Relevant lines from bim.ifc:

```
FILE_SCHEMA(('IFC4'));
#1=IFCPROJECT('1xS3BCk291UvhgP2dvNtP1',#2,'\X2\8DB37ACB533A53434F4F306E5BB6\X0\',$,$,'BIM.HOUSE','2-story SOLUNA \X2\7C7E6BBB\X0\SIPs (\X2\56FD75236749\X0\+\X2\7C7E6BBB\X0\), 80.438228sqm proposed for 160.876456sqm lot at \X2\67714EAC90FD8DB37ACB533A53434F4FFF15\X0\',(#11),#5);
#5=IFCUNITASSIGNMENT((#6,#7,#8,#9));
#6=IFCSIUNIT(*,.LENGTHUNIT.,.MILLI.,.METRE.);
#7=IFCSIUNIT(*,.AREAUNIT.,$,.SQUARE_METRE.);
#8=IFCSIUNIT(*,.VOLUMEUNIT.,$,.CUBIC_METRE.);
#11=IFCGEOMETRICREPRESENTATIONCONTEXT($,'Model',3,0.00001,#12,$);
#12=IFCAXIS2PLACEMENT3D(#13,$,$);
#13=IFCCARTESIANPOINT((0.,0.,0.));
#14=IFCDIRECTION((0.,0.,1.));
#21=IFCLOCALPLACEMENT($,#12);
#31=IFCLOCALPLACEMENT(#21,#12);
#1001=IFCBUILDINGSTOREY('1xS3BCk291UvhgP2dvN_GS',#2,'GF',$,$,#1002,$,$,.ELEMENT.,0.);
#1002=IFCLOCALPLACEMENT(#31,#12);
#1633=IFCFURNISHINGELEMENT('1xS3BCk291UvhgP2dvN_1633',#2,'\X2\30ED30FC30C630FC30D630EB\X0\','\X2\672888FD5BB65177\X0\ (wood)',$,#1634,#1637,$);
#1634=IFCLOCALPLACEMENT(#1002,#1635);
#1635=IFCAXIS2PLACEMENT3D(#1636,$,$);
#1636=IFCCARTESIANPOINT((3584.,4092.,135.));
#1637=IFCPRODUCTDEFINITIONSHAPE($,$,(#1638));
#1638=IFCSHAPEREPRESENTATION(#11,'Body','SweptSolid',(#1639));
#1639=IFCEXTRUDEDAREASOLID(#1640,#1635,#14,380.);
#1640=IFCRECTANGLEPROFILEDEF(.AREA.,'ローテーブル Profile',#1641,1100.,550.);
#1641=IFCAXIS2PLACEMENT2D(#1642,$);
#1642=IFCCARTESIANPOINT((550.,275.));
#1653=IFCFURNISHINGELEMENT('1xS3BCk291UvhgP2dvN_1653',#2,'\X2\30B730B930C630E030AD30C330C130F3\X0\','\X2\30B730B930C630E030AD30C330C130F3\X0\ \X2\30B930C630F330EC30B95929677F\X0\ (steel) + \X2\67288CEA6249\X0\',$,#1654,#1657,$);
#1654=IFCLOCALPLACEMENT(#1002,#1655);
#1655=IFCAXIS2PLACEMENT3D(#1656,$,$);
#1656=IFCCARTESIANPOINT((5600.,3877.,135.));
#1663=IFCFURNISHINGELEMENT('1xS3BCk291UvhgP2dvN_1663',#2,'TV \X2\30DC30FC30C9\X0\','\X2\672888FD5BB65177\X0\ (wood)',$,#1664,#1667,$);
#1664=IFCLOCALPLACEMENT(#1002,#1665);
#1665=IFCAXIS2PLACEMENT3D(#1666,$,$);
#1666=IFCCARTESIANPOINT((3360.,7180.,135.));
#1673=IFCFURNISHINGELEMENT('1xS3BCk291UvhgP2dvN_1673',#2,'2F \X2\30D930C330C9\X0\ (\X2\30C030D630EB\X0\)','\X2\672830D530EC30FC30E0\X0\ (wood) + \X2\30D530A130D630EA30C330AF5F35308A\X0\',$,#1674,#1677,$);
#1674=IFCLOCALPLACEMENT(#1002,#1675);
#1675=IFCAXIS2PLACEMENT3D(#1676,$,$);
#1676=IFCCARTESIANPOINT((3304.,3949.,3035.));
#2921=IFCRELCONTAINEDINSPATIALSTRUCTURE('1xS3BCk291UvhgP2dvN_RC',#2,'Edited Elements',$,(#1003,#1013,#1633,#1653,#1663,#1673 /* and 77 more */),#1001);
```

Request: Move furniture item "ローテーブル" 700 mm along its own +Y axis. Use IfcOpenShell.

```python
import ifcopenshell
import ifcopenshell.api.geometry
import ifcopenshell.util.placement
import ifcopenshell.util.unit

model = ifcopenshell.open("bim.ifc")
unit_scale = ifcopenshell.util.unit.calculate_unit_scale(model)

item = model.by_id(1633)
matrix = ifcopenshell.util.placement.get_local_placement(item.ObjectPlacement)
matrix[:3, 3] += matrix[:3, 1] * 0.7 / unit_scale
ifcopenshell.api.geometry.edit_object_placement(model, product=item, matrix=matrix, is_si=False)

print(ifcopenshell.util.placement.get_local_placement(item.ObjectPlacement).round(3) + 0.0)

model.write("bim_updated.ifc")
```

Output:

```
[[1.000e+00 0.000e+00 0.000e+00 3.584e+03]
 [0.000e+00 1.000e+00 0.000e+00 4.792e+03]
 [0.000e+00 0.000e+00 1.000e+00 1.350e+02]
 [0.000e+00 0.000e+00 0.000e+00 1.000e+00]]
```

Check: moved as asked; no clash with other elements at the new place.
